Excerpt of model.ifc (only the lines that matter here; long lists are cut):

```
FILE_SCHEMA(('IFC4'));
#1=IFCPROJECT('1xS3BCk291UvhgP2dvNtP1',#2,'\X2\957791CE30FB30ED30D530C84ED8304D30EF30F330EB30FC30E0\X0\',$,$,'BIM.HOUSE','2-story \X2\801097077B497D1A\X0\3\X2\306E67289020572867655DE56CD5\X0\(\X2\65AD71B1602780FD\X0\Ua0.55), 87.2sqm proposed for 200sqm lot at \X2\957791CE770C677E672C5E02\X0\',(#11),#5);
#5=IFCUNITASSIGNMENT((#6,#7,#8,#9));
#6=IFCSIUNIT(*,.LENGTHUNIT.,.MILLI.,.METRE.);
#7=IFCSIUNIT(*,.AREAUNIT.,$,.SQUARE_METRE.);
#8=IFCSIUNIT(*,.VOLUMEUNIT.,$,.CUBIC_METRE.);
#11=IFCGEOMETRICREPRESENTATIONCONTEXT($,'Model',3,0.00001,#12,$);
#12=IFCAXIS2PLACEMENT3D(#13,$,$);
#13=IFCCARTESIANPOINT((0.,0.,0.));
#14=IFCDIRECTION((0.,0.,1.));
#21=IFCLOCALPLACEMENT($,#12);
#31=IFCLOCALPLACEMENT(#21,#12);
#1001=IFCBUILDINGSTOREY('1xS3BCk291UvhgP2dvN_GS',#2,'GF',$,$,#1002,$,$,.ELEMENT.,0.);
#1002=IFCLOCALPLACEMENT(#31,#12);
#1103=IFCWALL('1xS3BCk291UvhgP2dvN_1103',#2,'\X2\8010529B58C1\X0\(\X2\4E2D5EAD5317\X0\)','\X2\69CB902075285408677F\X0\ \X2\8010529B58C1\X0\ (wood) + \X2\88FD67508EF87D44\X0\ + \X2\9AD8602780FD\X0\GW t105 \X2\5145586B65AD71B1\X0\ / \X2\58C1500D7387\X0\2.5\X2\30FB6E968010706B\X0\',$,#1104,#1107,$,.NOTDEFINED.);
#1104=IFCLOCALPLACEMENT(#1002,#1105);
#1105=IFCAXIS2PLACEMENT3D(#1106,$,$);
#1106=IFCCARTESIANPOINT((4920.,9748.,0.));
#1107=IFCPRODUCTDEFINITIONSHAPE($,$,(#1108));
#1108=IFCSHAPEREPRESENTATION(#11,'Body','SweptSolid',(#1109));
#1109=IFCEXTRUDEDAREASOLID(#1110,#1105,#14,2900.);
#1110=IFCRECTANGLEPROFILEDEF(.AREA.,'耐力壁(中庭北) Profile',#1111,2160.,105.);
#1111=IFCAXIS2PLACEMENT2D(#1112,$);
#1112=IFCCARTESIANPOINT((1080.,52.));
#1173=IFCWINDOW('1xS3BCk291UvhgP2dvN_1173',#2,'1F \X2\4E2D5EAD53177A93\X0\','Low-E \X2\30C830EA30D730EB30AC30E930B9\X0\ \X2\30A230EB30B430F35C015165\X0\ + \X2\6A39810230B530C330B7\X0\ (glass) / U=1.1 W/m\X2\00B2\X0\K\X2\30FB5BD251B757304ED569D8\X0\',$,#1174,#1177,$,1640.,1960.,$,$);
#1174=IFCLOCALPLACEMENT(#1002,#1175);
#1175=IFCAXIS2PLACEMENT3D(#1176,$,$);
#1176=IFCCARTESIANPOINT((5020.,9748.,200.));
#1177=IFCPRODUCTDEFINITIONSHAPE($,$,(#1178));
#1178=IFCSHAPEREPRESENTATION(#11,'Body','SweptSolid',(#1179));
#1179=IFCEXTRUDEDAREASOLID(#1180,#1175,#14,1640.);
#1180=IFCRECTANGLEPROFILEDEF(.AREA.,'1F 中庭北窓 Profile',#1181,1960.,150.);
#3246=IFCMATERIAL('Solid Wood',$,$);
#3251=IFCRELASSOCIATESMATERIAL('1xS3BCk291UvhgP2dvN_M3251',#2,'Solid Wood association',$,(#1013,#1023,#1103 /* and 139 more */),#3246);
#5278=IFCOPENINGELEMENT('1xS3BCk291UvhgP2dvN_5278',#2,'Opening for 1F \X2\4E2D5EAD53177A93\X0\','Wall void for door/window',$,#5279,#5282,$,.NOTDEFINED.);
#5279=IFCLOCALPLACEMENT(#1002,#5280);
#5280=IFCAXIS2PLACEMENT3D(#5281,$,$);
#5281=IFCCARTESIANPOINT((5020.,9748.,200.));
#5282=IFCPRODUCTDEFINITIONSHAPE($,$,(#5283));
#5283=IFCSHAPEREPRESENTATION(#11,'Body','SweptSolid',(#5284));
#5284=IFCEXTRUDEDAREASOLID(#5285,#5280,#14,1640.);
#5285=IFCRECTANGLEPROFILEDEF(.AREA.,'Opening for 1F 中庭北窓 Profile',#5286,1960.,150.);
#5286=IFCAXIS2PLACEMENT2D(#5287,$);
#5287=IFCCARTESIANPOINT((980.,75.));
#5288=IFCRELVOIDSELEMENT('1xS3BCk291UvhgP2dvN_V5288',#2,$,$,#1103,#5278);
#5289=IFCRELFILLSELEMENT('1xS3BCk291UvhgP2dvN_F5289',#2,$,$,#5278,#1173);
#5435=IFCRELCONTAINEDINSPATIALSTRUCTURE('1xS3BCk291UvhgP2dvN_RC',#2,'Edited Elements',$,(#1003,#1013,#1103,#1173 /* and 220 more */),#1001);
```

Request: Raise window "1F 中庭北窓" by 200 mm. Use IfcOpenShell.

```python
import numpy as np
import ifcopenshell
import ifcopenshell.api.geometry
import ifcopenshell.util.placement
import ifcopenshell.util.unit

model = ifcopenshell.open("model.ifc")
unit_scale = ifcopenshell.util.unit.calculate_unit_scale(model)

window = model.by_guid("1xS3BCk291UvhgP2dvN_1173")
opening = window.FillsVoids[0].RelatingOpeningElement
dz = 200.0

shift = np.array([0.0, 0.0, dz])
# The window is not placed relative to its opening, so move both.
for product in (opening, window):
    matrix = ifcopenshell.util.placement.get_local_placement(product.ObjectPlacement)
    matrix[:3, 3] += shift
    ifcopenshell.api.geometry.edit_object_placement(model, product=product, matrix=matrix, is_si=False)

print(f"moved by {dz * unit_scale:+.3f} m")

model.write("model_v2.ifc")
```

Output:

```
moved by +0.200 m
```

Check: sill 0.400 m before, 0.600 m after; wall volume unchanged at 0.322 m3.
